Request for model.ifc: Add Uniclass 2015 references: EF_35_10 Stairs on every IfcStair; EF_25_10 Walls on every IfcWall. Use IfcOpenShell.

First a look at what the model holds.

```python
import ifcopenshell

model = ifcopenshell.open("model.ifc")
print(model.schema)
print("classifications:", [c.Name for c in model.by_type("IfcClassification")])
for ifc_class in ("IfcDoor", "IfcRoof", "IfcStair", "IfcWall", "IfcWindow"):
    print(ifc_class, len(model.by_type(ifc_class)))
```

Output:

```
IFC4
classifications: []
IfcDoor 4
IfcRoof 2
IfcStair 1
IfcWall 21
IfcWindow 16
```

```python
import ifcopenshell
import ifcopenshell.api.classification

model = ifcopenshell.open("model.ifc")

system = ifcopenshell.api.classification.add_classification(model, classification="Uniclass 2015")

codes = {
    "IfcStair": ("EF_35_10", "Stairs"),
    "IfcWall": ("EF_25_10", "Walls"),
}
for ifc_class, (code, name) in codes.items():
    products = model.by_type(ifc_class)
    ifcopenshell.api.classification.add_reference(
        model, products=products, classification=system, identification=code, name=name
    )
    print(code, len(products))

model.write("model_edited.ifc")
```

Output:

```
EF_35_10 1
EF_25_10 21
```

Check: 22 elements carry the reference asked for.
